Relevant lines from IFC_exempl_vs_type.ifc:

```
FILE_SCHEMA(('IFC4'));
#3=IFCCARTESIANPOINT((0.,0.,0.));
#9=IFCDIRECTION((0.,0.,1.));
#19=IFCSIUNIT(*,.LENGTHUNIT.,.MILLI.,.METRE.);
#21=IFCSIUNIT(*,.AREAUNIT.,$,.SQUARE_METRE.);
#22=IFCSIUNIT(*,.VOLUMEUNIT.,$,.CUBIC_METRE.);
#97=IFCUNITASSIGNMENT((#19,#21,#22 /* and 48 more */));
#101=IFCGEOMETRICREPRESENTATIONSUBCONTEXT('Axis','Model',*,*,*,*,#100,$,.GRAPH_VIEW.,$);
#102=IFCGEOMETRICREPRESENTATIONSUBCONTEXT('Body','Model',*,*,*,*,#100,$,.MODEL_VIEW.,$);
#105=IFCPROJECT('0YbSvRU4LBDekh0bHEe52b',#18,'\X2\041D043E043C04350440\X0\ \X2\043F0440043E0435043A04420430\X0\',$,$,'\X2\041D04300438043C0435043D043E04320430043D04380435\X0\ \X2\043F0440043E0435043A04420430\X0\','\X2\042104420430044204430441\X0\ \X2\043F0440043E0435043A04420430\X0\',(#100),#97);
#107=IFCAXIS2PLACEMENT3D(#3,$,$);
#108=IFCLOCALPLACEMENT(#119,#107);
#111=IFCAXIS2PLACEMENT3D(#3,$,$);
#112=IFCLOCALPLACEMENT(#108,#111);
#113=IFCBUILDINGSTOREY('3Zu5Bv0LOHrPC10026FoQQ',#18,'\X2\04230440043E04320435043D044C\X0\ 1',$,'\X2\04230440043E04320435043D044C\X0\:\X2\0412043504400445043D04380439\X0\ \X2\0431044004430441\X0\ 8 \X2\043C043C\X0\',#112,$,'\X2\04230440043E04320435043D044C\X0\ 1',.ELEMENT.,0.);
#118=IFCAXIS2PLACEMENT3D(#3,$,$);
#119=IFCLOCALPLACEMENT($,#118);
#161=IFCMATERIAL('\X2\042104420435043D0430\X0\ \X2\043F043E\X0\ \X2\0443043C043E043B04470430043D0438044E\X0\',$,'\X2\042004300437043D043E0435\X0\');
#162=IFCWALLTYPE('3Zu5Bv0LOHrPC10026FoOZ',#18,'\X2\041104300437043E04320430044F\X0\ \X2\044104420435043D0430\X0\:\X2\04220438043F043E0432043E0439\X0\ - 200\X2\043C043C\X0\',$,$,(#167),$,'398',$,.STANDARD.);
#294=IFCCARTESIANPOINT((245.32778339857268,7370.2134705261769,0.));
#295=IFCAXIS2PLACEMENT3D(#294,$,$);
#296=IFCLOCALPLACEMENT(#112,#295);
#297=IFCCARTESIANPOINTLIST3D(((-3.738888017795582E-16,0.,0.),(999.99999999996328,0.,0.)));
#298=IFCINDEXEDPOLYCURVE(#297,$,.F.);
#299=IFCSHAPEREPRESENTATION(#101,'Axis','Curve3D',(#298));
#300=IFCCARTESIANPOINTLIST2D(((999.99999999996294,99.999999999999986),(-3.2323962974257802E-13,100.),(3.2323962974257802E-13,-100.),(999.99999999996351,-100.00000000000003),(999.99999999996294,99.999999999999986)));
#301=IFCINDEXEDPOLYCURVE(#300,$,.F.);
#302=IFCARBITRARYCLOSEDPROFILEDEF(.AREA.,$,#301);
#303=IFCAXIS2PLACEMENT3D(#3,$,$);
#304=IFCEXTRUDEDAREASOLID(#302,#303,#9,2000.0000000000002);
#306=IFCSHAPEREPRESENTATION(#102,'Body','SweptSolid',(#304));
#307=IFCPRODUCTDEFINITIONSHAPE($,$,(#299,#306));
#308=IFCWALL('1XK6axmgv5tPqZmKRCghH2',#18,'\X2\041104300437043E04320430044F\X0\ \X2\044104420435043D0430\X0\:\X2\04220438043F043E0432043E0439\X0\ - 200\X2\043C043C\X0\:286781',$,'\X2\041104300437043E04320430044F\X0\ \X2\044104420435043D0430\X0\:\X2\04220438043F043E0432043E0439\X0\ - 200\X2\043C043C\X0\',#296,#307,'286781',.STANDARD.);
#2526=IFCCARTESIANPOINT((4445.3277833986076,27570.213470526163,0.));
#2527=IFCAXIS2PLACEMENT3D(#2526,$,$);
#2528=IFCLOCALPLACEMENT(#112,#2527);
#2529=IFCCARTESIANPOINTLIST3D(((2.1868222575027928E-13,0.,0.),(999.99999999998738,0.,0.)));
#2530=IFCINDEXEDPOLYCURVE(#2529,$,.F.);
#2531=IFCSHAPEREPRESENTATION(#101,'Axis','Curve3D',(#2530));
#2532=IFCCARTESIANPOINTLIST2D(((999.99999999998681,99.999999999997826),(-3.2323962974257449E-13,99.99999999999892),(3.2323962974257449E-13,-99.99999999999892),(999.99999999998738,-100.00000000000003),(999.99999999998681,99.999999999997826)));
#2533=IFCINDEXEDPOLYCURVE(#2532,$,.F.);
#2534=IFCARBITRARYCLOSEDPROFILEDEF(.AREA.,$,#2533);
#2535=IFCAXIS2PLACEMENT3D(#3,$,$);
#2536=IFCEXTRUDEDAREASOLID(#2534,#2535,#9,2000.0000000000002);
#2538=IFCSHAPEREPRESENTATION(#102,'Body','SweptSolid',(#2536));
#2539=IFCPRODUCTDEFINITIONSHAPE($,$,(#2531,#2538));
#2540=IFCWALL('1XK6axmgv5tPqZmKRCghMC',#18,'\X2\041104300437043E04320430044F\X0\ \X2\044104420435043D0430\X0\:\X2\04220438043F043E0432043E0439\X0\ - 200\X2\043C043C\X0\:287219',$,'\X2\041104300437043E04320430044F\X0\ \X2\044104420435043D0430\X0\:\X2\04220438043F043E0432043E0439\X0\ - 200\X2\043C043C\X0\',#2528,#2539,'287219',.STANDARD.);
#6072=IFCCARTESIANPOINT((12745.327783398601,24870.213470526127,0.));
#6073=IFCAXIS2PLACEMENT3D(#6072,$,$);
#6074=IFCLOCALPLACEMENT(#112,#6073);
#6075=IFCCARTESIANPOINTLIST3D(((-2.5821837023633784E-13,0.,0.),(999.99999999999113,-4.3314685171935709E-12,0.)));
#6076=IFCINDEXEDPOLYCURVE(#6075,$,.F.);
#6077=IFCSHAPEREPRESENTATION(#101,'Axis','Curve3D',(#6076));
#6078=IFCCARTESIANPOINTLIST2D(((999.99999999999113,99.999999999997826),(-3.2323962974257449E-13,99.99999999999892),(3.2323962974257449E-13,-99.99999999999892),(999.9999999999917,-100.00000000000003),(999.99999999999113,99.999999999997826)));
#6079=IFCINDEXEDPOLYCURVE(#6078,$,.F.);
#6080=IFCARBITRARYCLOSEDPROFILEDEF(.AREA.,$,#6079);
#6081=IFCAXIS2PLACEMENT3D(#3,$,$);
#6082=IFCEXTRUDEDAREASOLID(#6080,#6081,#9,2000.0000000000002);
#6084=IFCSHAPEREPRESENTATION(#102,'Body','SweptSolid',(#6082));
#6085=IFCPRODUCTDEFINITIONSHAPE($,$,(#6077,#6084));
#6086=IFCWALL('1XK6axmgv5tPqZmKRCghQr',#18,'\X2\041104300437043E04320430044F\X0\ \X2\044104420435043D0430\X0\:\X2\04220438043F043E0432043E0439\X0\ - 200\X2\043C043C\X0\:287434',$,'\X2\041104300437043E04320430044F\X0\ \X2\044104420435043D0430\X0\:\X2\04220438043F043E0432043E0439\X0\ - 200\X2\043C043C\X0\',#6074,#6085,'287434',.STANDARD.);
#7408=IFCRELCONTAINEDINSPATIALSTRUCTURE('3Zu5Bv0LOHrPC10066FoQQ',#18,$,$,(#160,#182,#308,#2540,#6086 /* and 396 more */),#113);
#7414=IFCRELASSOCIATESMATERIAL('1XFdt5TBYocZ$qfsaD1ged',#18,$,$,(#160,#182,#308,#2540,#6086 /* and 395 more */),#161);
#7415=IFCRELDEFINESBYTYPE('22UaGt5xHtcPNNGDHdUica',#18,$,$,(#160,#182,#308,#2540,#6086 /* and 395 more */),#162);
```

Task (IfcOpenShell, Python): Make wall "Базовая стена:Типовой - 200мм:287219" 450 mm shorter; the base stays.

```python
import ifcopenshell
import ifcopenshell.geom
import ifcopenshell.util.representation
import ifcopenshell.util.shape

model = ifcopenshell.open("IFC_exempl_vs_type.ifc")
settings = ifcopenshell.geom.settings()


def volume(element):
    """Net volume in cubic metres, openings subtracted."""
    shape = ifcopenshell.geom.create_shape(settings, element)
    return ifcopenshell.util.shape.get_volume(shape.geometry)


wall = model.by_guid("1XK6axmgv5tPqZmKRCghMC")
before = volume(wall)

body = ifcopenshell.util.representation.get_representation(wall, "Model", "Body")
solid = body.Items[0]
old_height = solid.Depth
solid.Depth -= 450.0
after = volume(wall)

print(f"height {old_height:g} -> {solid.Depth:g}, volume {before:.3f} -> {after:.3f} m3")

model.write("IFC_exempl_vs_type_rev.ifc")
```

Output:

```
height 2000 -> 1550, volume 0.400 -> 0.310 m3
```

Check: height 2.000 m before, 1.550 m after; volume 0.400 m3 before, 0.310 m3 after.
